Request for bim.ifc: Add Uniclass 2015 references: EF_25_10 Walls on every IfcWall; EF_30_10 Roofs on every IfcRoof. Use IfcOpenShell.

First a look at what the model holds.

```python
import ifcopenshell

model = ifcopenshell.open("bim.ifc")
print(model.schema)
print("classifications:", [c.Name for c in model.by_type("IfcClassification")])
for ifc_class in ("IfcDoor", "IfcRoof", "IfcStair", "IfcWall", "IfcWindow"):
    print(ifc_class, len(model.by_type(ifc_class)))
```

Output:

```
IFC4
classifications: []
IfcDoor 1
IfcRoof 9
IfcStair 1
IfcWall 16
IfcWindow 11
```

```python
import ifcopenshell
import ifcopenshell.api.classification

model = ifcopenshell.open("bim.ifc")

system = ifcopenshell.api.classification.add_classification(model, classification="Uniclass 2015")

codes = {
    "IfcWall": ("EF_25_10", "Walls"),
    "IfcRoof": ("EF_30_10", "Roofs"),
}
for ifc_class, (code, name) in codes.items():
    products = model.by_type(ifc_class)
    ifcopenshell.api.classification.add_reference(
        model, products=products, classification=system, identification=code, name=name
    )
    print(code, len(products))

model.write("bim-out.ifc")
```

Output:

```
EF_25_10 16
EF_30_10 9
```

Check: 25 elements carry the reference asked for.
